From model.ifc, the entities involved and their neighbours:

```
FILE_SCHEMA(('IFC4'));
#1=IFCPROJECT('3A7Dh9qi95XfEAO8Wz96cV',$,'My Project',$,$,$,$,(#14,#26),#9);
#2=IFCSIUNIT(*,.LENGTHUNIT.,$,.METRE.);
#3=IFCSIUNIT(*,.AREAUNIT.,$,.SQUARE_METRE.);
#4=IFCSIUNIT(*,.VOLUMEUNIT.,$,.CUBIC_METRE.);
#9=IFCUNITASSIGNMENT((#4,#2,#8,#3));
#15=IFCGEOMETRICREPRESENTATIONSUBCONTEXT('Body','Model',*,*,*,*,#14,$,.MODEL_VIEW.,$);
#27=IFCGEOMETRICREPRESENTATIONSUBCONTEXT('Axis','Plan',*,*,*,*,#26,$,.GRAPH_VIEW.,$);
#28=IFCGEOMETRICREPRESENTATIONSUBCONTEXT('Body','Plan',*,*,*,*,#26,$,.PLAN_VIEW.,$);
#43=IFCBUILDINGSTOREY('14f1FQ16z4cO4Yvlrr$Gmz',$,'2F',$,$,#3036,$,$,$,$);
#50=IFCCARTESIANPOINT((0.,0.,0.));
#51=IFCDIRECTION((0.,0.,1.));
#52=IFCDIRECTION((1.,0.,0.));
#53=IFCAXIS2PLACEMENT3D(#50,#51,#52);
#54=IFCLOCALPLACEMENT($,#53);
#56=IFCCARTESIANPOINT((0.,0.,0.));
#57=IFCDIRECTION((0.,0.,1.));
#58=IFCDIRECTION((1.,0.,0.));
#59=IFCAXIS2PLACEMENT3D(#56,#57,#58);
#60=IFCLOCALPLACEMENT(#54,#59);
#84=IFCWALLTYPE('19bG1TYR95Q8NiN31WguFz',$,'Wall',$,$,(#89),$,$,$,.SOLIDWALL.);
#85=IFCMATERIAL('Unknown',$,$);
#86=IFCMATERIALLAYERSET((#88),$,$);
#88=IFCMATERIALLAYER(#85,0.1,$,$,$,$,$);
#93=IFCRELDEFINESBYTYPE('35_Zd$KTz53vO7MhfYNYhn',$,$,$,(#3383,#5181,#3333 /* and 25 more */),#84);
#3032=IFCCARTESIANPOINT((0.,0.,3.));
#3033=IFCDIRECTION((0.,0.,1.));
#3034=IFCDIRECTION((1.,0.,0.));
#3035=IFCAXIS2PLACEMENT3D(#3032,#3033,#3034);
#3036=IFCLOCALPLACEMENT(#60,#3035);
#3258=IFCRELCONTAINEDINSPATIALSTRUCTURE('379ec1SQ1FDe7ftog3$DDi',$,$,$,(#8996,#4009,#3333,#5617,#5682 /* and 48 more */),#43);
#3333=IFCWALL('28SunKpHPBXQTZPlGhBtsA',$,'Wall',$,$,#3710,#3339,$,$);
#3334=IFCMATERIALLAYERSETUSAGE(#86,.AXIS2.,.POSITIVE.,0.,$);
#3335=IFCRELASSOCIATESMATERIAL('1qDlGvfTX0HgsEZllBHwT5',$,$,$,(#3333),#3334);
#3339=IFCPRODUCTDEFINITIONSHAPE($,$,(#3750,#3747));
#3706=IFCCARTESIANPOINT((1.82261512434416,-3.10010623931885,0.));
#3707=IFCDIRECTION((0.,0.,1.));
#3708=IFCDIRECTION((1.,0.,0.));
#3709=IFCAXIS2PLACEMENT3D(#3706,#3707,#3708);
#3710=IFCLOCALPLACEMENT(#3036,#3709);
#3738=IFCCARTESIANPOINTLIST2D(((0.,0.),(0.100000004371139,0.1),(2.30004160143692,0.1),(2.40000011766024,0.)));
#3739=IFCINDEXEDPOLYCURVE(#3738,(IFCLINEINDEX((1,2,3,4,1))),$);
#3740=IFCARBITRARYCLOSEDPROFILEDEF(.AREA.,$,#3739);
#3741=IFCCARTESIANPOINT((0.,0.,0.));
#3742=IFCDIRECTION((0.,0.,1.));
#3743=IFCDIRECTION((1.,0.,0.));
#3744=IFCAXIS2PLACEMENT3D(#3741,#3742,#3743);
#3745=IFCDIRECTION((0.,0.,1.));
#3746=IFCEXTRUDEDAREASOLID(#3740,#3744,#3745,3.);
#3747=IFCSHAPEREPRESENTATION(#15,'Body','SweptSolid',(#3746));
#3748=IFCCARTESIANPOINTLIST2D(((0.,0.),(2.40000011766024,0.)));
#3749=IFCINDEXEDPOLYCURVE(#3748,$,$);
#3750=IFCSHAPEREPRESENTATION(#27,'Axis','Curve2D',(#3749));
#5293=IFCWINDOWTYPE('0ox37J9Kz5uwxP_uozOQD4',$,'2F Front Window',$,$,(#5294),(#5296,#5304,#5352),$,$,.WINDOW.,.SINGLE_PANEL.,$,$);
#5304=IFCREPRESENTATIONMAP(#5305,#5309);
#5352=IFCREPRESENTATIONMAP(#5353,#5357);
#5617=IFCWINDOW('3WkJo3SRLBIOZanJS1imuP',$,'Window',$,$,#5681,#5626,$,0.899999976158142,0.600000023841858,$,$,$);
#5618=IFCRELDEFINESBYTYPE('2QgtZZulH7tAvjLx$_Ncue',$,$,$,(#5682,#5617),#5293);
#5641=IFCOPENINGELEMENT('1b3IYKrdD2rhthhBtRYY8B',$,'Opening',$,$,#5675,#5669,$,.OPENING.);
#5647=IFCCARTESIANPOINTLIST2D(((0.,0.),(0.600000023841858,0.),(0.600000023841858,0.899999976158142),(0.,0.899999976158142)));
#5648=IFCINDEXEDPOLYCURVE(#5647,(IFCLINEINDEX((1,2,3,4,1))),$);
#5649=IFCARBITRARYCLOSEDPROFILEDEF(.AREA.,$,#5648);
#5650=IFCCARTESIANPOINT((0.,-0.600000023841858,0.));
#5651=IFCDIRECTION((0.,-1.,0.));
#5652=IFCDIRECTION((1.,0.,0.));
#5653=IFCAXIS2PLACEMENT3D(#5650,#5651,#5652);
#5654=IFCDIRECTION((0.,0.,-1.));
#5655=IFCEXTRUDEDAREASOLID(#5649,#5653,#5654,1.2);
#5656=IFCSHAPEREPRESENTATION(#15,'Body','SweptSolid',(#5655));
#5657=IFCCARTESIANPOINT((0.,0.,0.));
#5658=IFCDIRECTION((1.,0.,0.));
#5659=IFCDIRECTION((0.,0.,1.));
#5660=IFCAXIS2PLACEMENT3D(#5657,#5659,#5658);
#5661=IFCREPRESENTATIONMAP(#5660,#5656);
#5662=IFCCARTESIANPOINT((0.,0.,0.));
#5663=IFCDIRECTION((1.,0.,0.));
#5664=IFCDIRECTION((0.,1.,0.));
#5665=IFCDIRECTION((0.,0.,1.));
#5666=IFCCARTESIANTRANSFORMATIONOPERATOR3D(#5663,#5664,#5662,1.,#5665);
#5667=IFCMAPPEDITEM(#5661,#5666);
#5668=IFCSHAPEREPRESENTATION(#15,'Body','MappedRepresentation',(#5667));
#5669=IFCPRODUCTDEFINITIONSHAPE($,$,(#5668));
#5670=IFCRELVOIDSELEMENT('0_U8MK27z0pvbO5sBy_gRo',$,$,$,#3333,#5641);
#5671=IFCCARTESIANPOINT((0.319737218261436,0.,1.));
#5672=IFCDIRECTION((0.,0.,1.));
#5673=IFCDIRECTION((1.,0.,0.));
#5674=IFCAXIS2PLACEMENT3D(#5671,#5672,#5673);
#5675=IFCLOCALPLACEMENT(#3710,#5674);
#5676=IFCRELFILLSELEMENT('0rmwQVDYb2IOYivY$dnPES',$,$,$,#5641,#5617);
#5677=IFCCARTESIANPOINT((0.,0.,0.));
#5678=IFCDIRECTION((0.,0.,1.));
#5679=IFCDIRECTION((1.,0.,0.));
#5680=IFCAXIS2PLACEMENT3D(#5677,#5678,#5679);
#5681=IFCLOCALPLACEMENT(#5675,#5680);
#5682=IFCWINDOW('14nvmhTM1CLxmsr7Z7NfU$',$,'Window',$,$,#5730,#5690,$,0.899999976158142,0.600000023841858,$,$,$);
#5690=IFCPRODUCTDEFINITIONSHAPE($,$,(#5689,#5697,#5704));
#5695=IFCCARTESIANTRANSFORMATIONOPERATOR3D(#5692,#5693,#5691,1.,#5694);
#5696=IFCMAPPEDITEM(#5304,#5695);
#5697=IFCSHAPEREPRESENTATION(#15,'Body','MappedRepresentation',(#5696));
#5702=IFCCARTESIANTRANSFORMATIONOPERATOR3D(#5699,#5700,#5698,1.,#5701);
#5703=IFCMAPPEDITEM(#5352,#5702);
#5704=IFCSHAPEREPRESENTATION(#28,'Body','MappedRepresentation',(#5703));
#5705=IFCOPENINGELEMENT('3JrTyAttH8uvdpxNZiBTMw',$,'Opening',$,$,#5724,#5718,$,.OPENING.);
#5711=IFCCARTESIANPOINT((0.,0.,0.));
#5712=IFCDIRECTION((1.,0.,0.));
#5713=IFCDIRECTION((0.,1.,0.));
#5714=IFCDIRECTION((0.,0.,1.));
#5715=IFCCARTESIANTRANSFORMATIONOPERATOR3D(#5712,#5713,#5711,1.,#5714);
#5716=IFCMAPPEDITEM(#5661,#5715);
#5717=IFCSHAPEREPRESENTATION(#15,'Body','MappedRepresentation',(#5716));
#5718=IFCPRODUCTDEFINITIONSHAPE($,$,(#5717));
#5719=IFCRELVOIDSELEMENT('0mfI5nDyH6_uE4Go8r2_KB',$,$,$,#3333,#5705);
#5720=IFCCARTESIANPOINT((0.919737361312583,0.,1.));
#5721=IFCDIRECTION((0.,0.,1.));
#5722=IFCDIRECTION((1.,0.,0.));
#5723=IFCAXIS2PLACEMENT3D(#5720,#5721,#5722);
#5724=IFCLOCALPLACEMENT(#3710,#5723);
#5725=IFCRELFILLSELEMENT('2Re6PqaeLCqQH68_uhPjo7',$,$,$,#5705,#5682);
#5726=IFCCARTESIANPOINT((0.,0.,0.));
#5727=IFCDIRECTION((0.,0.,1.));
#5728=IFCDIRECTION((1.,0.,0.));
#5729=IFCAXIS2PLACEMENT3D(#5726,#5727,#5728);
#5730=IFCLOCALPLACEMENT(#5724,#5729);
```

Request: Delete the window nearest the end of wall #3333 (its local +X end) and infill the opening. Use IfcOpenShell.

```python
import ifcopenshell
import ifcopenshell.api.feature
import ifcopenshell.api.root
import ifcopenshell.geom
import ifcopenshell.util.shape

model = ifcopenshell.open("model.ifc")
settings = ifcopenshell.geom.settings()


def volume(element):
    """Net volume in cubic metres, openings subtracted."""
    shape = ifcopenshell.geom.create_shape(settings, element)
    return ifcopenshell.util.shape.get_volume(shape.geometry)


window = model.by_guid("14nvmhTM1CLxmsr7Z7NfU$")
opening = window.FillsVoids[0].RelatingOpeningElement
wall = opening.VoidsElements[0].RelatingBuildingElement
before = volume(wall)

ifcopenshell.api.root.remove_product(model, product=window)
ifcopenshell.api.feature.remove_feature(model, feature=opening)

after = volume(wall)

print(f"wall volume {before:.3f} -> {after:.3f} m3")

model.write("model-out.ifc")
```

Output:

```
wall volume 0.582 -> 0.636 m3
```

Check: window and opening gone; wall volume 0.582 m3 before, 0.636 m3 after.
